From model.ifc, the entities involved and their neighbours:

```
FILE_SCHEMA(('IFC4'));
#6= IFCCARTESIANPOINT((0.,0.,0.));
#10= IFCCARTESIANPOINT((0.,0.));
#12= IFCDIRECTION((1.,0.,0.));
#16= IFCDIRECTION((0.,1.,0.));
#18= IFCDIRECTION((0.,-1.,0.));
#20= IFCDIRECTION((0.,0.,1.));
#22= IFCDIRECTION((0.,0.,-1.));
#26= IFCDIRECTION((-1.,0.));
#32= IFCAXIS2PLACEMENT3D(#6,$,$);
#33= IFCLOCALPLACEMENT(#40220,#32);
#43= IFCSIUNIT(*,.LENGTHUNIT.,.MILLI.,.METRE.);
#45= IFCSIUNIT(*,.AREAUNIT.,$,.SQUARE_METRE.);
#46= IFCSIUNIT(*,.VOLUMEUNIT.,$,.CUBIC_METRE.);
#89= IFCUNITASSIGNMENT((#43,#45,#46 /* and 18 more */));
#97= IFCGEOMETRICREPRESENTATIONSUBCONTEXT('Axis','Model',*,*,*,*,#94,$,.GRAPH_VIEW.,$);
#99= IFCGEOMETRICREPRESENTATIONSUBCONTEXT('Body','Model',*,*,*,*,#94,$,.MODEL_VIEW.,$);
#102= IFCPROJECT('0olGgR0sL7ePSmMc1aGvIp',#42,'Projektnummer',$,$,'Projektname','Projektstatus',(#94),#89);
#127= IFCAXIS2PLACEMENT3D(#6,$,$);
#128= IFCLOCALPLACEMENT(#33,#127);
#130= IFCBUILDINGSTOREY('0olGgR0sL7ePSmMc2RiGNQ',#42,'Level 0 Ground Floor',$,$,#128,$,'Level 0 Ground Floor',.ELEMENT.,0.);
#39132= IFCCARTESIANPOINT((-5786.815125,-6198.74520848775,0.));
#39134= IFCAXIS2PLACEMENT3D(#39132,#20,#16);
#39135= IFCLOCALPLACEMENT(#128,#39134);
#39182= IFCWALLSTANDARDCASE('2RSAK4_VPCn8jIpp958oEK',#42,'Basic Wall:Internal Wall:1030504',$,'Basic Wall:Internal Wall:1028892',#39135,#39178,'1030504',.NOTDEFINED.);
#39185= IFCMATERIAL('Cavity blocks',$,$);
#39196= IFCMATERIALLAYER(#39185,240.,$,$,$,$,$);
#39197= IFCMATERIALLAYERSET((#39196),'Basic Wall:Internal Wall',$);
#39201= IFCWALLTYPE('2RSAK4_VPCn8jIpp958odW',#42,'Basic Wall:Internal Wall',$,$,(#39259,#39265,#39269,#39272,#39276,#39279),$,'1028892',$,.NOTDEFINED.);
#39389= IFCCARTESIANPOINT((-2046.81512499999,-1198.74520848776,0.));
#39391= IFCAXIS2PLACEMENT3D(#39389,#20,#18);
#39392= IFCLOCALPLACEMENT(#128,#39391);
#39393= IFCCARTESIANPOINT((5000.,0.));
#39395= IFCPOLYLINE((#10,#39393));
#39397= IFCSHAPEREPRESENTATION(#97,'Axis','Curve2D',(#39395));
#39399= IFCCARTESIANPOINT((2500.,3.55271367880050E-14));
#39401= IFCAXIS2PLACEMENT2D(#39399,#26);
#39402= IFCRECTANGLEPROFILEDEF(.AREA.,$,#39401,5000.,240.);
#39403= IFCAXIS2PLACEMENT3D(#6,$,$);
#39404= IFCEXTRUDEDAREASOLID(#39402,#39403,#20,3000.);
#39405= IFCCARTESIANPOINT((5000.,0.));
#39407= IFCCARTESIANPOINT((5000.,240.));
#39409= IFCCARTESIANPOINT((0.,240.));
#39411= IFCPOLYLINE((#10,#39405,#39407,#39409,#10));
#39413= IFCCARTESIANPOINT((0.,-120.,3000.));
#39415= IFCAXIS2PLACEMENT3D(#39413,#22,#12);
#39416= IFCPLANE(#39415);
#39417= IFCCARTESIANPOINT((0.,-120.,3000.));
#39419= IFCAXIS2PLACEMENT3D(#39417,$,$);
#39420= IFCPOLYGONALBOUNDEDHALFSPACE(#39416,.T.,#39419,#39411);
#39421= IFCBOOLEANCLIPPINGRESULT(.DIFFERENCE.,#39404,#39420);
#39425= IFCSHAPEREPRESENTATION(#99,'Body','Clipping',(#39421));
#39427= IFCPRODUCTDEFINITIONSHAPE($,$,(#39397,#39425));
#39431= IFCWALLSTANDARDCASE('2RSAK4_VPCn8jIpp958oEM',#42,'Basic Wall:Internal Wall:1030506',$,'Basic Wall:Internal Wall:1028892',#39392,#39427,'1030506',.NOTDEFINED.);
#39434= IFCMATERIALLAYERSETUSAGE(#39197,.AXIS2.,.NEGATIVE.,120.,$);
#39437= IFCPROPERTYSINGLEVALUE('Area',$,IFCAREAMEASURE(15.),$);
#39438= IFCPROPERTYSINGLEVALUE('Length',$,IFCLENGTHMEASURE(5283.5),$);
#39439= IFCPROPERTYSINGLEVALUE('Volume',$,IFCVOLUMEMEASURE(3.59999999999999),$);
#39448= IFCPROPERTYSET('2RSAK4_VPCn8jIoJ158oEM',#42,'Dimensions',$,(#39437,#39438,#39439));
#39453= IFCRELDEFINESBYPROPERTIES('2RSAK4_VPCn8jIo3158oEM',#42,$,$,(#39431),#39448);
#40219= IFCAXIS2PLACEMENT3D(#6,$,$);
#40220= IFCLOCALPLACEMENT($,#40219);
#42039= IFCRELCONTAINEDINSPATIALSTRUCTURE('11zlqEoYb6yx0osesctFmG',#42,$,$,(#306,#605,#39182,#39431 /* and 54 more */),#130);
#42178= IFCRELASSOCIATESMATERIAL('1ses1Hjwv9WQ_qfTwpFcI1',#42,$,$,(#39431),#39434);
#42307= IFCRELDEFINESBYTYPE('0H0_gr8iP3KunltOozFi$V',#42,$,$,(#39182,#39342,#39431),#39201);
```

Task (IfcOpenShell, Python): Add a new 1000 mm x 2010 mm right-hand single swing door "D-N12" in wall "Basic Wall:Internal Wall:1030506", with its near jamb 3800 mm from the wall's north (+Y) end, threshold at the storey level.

```python
import numpy as np
import ifcopenshell
import ifcopenshell.api.feature
import ifcopenshell.api.geometry
import ifcopenshell.api.pset
import ifcopenshell.api.root
import ifcopenshell.api.spatial
import ifcopenshell.geom
import ifcopenshell.util.element
import ifcopenshell.util.placement
import ifcopenshell.util.representation
import ifcopenshell.util.shape
import ifcopenshell.util.unit

model = ifcopenshell.open("model.ifc")
unit_scale = ifcopenshell.util.unit.calculate_unit_scale(model)
area_scale = ifcopenshell.util.unit.calculate_unit_scale(model, "AREAUNIT")
volume_scale = ifcopenshell.util.unit.calculate_unit_scale(model, "VOLUMEUNIT")
settings = ifcopenshell.geom.settings()


def volume(element):
    """Net volume in cubic metres, openings subtracted."""
    shape = ifcopenshell.geom.create_shape(settings, element)
    return ifcopenshell.util.shape.get_volume(shape.geometry)


wall = model.by_guid("2RSAK4_VPCn8jIpp958oEM")
storey = ifcopenshell.util.element.get_container(wall, ifc_class="IfcBuildingStorey")
context = ifcopenshell.util.representation.get_context(model, "Model", "Body", "MODEL_VIEW")
before = volume(wall)

width, height, from_end, sill = 1, 2.01, 3.8, 0.0  # metres

# The wall runs along its own X axis, and the end named is its -X end.
wall_shape = ifcopenshell.geom.create_shape(settings, wall)
x, y, z = ifcopenshell.util.shape.get_vertices(wall_shape.geometry).T
start = x.min() + from_end
face, thickness = float(y.min()), float(y.max() - y.min())
wall_matrix = ifcopenshell.util.placement.get_local_placement(wall.ObjectPlacement)
level = ifcopenshell.util.placement.get_local_placement(storey.ObjectPlacement)[2, 3]


def in_wall(x, y):
    """Placement at x, y metres in the wall's axes, at sill height."""
    matrix = wall_matrix.copy()
    matrix[:, 3] = wall_matrix @ np.array([x / unit_scale, y / unit_scale, 0.0, 1.0])
    matrix[2, 3] = level + sill / unit_scale
    return matrix


# Opening: a box that overshoots both wall faces by 50 mm.
opening = ifcopenshell.api.root.create_entity(model, ifc_class="IfcOpeningElement", predefined_type="OPENING")
box = ifcopenshell.api.geometry.add_wall_representation(
    model, context=context, length=width, height=height, thickness=thickness + 0.1
)
ifcopenshell.api.geometry.assign_representation(model, product=opening, representation=box)
ifcopenshell.api.geometry.edit_object_placement(model, product=opening, matrix=in_wall(start, face - 0.05), is_si=False)
ifcopenshell.api.feature.add_feature(model, feature=opening, element=wall)

door = ifcopenshell.api.root.create_entity(model, ifc_class="IfcDoor", name="D-N12", predefined_type="DOOR")
door.OverallWidth, door.OverallHeight = width / unit_scale, height / unit_scale
door.OperationType = "SINGLE_SWING_RIGHT"
body = ifcopenshell.api.geometry.add_door_representation(
    model,
    context=context,
    overall_width=door.OverallWidth,
    overall_height=door.OverallHeight,
    operation_type="SINGLE_SWING_RIGHT",
    lining_properties={"LiningDepth": thickness / unit_scale, "ThresholdDepth": thickness / unit_scale},
)
ifcopenshell.api.geometry.assign_representation(model, product=door, representation=body)
ifcopenshell.api.spatial.assign_container(model, products=[door], relating_structure=storey)
ifcopenshell.api.feature.add_filling(model, opening=opening, element=door)

# The lining spans the wall, so the door starts at the wall face.
ifcopenshell.api.geometry.edit_object_placement(model, product=door, matrix=in_wall(start, face), is_si=False)

after = volume(wall)

# Update the wall's stored quantities.
pset = model.by_id(ifcopenshell.util.element.get_pset(wall, "Dimensions", should_inherit=False)["id"])
ifcopenshell.api.pset.edit_pset(model, pset=pset, properties={
    "Area": model.create_entity("IfcAreaMeasure", after / thickness / area_scale),
    "Volume": model.create_entity("IfcVolumeMeasure", after / volume_scale),
})

print(f"wall volume {before:.3f} -> {after:.3f} m3")

model.write("model_v2.ifc")
```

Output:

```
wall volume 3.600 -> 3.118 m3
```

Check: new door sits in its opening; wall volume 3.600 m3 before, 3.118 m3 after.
